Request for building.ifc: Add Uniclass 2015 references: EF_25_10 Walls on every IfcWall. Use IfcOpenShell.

First a look at what the model holds.

```python
import ifcopenshell

model = ifcopenshell.open("building.ifc")
print(model.schema)
print("classifications:", [c.Name for c in model.by_type("IfcClassification")])
for ifc_class in ("IfcDoor", "IfcRoof", "IfcStair", "IfcWall", "IfcWindow"):
    print(ifc_class, len(model.by_type(ifc_class)))
```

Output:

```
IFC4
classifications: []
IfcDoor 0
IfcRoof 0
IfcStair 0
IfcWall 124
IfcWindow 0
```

```python
import ifcopenshell
import ifcopenshell.api.classification

model = ifcopenshell.open("building.ifc")

system = ifcopenshell.api.classification.add_classification(model, classification="Uniclass 2015")

codes = {
    "IfcWall": ("EF_25_10", "Walls"),
}
for ifc_class, (code, name) in codes.items():
    products = model.by_type(ifc_class)
    ifcopenshell.api.classification.add_reference(
        model, products=products, classification=system, identification=code, name=name
    )
    print(code, len(products))

model.write("building_updated.ifc")
```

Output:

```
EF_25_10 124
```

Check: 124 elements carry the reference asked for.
